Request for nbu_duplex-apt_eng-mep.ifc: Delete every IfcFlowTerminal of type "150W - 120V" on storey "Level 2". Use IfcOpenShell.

First a look at what the model holds.

```python
import ifcopenshell
import ifcopenshell.util.element

model = ifcopenshell.open("nbu_duplex-apt_eng-mep.ifc")
print(model.schema)
storey = next(s for s in model.by_type("IfcBuildingStorey") if s.Name == "Level 2")
terminals = [e for e in ifcopenshell.util.element.get_decomposition(storey) if e.is_a("IfcFlowTerminal")]
seen = {}
for e in terminals:
    element_type = ifcopenshell.util.element.get_type(e)
    name = element_type.Name if element_type not in (None, e) else None
    seen[name] = seen.get(name, 0) + 1
for name, count in sorted(seen.items(), key=str):
    print(count, "x", name)
```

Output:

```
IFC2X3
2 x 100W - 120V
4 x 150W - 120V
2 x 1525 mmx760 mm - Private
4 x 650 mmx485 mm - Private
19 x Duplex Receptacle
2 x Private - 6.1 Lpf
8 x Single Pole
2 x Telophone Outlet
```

```python
import ifcopenshell
import ifcopenshell.api.root
import ifcopenshell.util.element

model = ifcopenshell.open("nbu_duplex-apt_eng-mep.ifc")

storey = next(s for s in model.by_type("IfcBuildingStorey") if s.Name == "Level 2")
terminals = [e for e in ifcopenshell.util.element.get_decomposition(storey) if e.is_a("IfcFlowTerminal")]
targets = [e for e in terminals if (t := ifcopenshell.util.element.get_type(e)) not in (None, e) and t.Name == "150W - 120V"]

for e in targets:
    ifcopenshell.api.root.remove_product(model, product=e)
print(len(targets), "removed")

model.write("nbu_duplex-apt_eng-mep_rev.ifc")
```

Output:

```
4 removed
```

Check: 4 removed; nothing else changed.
